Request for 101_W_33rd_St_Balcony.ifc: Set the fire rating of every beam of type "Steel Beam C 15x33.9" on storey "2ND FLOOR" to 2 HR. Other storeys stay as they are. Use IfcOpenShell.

First a look at what the model holds.

```python
import ifcopenshell
import ifcopenshell.util.element

model = ifcopenshell.open("101_W_33rd_St_Balcony.ifc")
print(model.schema)
storey = next(s for s in model.by_type("IfcBuildingStorey") if s.Name == "2ND FLOOR")
beams = [e for e in ifcopenshell.util.element.get_decomposition(storey) if e.is_a("IfcBeam")]
seen = {}
for e in beams:
    element_type = ifcopenshell.util.element.get_type(e)
    key = (element_type.Name if element_type != e and element_type else None, ifcopenshell.util.element.get_pset(e, "Pset_BeamCommon", "FireRating"))
    seen[key] = seen.get(key, 0) + 1
for (name, value), count in sorted(seen.items(), key=str):
    print(count, "x", name, "|", value)
```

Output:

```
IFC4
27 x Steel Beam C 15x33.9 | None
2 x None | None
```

```python
import ifcopenshell
import ifcopenshell.api.pset
import ifcopenshell.util.element

model = ifcopenshell.open("101_W_33rd_St_Balcony.ifc")

storey = next(s for s in model.by_type("IfcBuildingStorey") if s.Name == "2ND FLOOR")
beams = [e for e in ifcopenshell.util.element.get_decomposition(storey) if e.is_a("IfcBeam")]

count = 0
for e in beams:
    element_type = ifcopenshell.util.element.get_type(e)
    if element_type in (None, e) or element_type.Name != "Steel Beam C 15x33.9":
        continue
    # add_pset returns the element's existing set when there is one.
    pset = ifcopenshell.api.pset.add_pset(model, product=e, name="Pset_BeamCommon")
    ifcopenshell.api.pset.edit_pset(model, pset=pset, properties={"FireRating": "2 HR"})
    count += 1

print(count, "beams updated")

model.write("101_W_33rd_St_Balcony_updated.ifc")
```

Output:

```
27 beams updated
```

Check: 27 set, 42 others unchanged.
